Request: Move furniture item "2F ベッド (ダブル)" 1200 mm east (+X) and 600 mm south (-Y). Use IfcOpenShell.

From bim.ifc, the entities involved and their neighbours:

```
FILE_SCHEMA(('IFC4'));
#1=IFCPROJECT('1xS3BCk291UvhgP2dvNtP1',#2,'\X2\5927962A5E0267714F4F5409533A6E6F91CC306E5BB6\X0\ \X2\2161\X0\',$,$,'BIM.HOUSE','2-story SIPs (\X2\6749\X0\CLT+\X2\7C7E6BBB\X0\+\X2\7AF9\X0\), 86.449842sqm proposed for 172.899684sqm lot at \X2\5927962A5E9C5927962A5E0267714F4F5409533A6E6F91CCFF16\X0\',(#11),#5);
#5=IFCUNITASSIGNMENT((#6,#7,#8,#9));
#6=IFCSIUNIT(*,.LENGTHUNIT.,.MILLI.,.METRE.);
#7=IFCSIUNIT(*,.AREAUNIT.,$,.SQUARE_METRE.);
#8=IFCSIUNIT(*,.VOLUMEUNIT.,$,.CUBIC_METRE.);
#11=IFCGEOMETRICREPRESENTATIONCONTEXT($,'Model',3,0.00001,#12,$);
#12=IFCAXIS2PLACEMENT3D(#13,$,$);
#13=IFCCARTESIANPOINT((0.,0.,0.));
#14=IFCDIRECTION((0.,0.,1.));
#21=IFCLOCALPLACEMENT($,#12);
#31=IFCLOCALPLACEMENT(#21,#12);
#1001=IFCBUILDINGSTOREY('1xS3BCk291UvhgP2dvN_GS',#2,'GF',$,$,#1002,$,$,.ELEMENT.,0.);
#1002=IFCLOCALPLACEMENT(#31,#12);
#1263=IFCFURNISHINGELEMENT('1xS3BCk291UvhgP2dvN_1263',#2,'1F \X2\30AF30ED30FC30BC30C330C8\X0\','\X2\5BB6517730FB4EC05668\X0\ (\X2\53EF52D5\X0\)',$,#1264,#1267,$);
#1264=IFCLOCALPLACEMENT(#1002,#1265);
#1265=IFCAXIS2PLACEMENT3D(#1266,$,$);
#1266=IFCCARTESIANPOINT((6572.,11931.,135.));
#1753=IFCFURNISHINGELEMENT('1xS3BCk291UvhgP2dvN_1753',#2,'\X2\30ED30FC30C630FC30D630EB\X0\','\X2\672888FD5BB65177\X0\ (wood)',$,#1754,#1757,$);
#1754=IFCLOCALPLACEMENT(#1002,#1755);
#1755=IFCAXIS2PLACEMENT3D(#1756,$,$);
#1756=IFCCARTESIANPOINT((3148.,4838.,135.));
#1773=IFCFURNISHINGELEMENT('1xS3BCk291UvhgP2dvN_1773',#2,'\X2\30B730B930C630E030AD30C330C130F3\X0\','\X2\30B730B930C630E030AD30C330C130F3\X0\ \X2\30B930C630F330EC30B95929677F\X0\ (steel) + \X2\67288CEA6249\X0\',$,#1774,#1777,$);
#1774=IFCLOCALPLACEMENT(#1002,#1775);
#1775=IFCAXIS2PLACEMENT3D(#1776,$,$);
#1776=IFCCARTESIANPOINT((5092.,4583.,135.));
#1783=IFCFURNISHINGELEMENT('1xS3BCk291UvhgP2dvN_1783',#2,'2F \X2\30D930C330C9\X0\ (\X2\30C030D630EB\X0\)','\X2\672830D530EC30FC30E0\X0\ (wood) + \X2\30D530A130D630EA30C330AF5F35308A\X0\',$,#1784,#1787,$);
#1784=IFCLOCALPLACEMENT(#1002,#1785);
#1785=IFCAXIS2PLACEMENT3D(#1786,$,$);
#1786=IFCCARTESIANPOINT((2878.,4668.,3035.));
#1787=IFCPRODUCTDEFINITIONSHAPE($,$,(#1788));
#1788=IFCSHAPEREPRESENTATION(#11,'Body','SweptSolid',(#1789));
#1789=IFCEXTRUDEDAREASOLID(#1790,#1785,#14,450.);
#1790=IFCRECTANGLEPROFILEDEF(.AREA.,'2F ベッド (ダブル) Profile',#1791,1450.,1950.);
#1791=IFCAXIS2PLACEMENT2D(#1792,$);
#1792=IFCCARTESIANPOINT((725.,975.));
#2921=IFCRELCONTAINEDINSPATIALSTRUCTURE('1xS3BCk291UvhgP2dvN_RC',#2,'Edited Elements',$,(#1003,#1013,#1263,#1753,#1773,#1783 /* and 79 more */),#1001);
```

```python
import ifcopenshell
import ifcopenshell.api.geometry
import ifcopenshell.util.placement
import ifcopenshell.util.unit

model = ifcopenshell.open("bim.ifc")
unit_scale = ifcopenshell.util.unit.calculate_unit_scale(model)

item = model.by_guid("1xS3BCk291UvhgP2dvN_1783")
matrix = ifcopenshell.util.placement.get_local_placement(item.ObjectPlacement)
matrix[0, 3] += 1.2 / unit_scale
matrix[1, 3] -= 0.6 / unit_scale
ifcopenshell.api.geometry.edit_object_placement(model, product=item, matrix=matrix, is_si=False)

print(ifcopenshell.util.placement.get_local_placement(item.ObjectPlacement).round(3) + 0.0)

model.write("bim_rev.ifc")
```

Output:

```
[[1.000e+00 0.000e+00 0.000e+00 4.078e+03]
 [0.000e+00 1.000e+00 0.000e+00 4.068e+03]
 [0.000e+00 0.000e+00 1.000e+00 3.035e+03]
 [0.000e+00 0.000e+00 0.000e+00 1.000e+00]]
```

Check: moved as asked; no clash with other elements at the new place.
